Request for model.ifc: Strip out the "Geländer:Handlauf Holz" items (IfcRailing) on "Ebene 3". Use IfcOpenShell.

First a look at what the model holds.

```python
import ifcopenshell
import ifcopenshell.util.element

model = ifcopenshell.open("model.ifc")
print(model.schema)
storey = next(s for s in model.by_type("IfcBuildingStorey") if s.Name == "Ebene 3")
railings = [e for e in ifcopenshell.util.element.get_decomposition(storey) if e.is_a("IfcRailing")]
seen = {}
for e in railings:
    element_type = ifcopenshell.util.element.get_type(e)
    name = element_type.Name if element_type not in (None, e) else None
    seen[name] = seen.get(name, 0) + 1
for name, count in sorted(seen.items(), key=str):
    print(count, "x", name)
```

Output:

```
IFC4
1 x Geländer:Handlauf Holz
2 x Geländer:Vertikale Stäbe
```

```python
import ifcopenshell
import ifcopenshell.api.root
import ifcopenshell.util.element

model = ifcopenshell.open("model.ifc")

storey = next(s for s in model.by_type("IfcBuildingStorey") if s.Name == "Ebene 3")
railings = [e for e in ifcopenshell.util.element.get_decomposition(storey) if e.is_a("IfcRailing")]
targets = [e for e in railings if (t := ifcopenshell.util.element.get_type(e)) not in (None, e) and t.Name == "Geländer:Handlauf Holz"]

for e in targets:
    ifcopenshell.api.root.remove_product(model, product=e)
print(len(targets), "removed")

model.write("model_v2.ifc")
```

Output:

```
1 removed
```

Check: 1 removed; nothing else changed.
